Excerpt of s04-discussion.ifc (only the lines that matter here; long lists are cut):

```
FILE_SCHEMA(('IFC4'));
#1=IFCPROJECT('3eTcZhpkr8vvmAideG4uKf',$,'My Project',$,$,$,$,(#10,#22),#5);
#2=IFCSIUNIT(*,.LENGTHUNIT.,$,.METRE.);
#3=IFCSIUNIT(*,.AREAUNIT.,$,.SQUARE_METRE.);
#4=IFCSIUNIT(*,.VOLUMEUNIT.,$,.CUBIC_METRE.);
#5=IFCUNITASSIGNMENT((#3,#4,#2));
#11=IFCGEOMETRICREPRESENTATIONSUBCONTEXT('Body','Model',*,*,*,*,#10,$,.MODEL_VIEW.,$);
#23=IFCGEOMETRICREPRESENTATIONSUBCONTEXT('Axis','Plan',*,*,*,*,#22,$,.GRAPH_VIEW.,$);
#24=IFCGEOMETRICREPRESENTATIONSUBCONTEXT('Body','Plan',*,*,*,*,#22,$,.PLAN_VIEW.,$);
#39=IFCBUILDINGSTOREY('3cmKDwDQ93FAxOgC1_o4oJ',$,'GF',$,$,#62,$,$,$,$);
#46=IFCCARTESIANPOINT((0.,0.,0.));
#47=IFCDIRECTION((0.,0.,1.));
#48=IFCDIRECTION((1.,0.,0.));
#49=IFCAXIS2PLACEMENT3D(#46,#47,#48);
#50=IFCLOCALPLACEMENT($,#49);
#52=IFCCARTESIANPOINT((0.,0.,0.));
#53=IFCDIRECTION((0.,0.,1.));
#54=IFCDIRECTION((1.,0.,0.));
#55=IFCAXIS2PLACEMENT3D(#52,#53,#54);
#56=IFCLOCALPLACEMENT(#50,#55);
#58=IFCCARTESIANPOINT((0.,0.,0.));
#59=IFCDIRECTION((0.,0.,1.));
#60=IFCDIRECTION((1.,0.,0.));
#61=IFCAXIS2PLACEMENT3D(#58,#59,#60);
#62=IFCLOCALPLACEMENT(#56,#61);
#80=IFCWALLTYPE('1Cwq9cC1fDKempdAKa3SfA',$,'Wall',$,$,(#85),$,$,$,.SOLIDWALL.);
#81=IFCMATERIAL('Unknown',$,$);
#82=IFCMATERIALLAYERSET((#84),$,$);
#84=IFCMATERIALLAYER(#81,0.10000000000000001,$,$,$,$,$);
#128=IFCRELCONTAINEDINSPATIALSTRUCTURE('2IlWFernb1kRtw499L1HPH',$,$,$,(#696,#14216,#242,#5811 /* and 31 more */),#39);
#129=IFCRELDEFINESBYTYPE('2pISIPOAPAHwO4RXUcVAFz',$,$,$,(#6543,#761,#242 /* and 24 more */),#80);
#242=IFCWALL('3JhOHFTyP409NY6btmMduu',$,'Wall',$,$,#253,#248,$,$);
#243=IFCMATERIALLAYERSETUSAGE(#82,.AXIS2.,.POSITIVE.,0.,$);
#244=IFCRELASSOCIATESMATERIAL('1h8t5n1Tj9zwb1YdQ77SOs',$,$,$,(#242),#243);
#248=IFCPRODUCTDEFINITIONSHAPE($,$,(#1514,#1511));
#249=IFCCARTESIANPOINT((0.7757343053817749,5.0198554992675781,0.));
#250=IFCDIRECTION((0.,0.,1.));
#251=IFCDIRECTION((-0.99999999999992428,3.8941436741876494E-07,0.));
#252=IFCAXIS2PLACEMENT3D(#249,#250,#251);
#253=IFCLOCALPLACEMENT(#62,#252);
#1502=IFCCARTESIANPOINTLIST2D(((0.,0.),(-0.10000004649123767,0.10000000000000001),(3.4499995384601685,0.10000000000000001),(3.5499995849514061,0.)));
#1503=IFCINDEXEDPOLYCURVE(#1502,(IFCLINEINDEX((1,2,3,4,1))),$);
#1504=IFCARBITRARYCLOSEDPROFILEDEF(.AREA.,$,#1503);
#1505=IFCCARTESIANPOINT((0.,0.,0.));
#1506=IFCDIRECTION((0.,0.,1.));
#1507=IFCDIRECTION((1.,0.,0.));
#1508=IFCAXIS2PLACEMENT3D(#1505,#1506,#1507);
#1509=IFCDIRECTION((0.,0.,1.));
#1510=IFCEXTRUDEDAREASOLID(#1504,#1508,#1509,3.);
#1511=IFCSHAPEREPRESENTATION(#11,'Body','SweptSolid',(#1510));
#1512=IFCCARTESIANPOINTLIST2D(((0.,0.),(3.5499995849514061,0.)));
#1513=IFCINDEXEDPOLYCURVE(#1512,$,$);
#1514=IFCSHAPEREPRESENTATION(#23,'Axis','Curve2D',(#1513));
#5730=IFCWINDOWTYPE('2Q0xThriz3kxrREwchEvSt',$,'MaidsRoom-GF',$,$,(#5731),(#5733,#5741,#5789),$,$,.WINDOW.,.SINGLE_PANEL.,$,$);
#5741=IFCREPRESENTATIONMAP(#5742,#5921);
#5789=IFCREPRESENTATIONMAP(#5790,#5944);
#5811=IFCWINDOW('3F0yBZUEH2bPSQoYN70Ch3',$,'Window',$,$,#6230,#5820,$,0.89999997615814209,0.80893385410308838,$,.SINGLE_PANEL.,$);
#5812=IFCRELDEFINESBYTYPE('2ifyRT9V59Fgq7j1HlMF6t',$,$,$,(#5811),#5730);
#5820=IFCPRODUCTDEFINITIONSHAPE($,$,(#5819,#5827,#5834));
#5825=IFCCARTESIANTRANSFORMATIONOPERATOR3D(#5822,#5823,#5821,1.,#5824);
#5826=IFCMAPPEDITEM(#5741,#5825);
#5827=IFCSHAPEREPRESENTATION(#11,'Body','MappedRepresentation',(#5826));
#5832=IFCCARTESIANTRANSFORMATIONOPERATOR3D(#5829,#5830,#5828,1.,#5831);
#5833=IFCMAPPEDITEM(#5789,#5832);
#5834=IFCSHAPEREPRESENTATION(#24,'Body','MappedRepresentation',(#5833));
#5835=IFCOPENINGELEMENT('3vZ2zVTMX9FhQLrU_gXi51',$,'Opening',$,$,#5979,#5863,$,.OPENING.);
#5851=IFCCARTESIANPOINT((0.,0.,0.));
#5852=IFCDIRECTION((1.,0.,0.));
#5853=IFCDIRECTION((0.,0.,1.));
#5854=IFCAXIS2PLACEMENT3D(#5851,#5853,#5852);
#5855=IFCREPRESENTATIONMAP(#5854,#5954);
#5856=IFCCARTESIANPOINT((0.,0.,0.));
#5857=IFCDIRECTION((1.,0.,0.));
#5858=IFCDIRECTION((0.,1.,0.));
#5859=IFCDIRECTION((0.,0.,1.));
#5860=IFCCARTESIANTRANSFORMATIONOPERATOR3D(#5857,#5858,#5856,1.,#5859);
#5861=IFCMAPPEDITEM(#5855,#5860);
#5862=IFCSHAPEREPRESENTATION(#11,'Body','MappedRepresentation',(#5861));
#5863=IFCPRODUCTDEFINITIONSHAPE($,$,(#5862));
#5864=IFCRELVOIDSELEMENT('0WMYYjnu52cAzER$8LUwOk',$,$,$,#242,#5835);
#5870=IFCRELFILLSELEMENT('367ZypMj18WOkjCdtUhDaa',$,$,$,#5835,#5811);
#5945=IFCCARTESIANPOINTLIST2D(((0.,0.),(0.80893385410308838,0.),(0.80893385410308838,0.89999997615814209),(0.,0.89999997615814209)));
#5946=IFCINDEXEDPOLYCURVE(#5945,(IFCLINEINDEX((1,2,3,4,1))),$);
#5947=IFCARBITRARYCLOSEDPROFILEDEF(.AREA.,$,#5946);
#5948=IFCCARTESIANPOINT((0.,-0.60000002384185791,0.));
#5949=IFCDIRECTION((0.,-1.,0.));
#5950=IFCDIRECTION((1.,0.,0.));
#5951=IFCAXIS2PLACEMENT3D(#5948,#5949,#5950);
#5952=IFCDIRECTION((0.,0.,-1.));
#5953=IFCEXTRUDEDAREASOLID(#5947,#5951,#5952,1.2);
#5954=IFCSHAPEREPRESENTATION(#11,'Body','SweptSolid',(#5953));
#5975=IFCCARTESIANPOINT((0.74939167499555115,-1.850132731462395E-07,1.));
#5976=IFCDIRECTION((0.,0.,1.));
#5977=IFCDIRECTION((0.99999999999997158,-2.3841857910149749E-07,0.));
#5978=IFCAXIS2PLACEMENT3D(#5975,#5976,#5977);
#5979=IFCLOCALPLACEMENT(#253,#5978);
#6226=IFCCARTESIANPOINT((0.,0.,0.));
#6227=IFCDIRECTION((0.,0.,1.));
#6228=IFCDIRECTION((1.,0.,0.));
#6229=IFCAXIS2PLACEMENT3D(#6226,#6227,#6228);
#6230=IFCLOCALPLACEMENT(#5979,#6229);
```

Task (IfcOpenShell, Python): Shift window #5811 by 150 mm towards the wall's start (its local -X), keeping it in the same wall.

```python
import ifcopenshell
import ifcopenshell.api.geometry
import ifcopenshell.util.placement

model = ifcopenshell.open("s04-discussion.ifc")

window = model.by_id(5811)
opening = window.FillsVoids[0].RelatingOpeningElement
wall = opening.VoidsElements[0].RelatingBuildingElement

wall_matrix = ifcopenshell.util.placement.get_local_placement(wall.ObjectPlacement)
shift = wall_matrix[:3, 0] * -0.15
before = ifcopenshell.util.placement.get_local_placement(window.ObjectPlacement)[:3, 3].copy()

# The window is placed relative to its opening, so it follows when the opening moves.
matrix = ifcopenshell.util.placement.get_local_placement(opening.ObjectPlacement)
matrix[:3, 3] += shift
ifcopenshell.api.geometry.edit_object_placement(
    model, product=opening, matrix=matrix, is_si=False, should_transform_children=True
)

after = ifcopenshell.util.placement.get_local_placement(window.ObjectPlacement)[:3, 3]
print("window moved by", (after - before).round(3) + 0.0)

model.write("s04-discussion_v2.ifc")
```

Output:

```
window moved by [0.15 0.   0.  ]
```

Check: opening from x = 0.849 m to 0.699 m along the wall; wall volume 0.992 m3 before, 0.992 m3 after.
